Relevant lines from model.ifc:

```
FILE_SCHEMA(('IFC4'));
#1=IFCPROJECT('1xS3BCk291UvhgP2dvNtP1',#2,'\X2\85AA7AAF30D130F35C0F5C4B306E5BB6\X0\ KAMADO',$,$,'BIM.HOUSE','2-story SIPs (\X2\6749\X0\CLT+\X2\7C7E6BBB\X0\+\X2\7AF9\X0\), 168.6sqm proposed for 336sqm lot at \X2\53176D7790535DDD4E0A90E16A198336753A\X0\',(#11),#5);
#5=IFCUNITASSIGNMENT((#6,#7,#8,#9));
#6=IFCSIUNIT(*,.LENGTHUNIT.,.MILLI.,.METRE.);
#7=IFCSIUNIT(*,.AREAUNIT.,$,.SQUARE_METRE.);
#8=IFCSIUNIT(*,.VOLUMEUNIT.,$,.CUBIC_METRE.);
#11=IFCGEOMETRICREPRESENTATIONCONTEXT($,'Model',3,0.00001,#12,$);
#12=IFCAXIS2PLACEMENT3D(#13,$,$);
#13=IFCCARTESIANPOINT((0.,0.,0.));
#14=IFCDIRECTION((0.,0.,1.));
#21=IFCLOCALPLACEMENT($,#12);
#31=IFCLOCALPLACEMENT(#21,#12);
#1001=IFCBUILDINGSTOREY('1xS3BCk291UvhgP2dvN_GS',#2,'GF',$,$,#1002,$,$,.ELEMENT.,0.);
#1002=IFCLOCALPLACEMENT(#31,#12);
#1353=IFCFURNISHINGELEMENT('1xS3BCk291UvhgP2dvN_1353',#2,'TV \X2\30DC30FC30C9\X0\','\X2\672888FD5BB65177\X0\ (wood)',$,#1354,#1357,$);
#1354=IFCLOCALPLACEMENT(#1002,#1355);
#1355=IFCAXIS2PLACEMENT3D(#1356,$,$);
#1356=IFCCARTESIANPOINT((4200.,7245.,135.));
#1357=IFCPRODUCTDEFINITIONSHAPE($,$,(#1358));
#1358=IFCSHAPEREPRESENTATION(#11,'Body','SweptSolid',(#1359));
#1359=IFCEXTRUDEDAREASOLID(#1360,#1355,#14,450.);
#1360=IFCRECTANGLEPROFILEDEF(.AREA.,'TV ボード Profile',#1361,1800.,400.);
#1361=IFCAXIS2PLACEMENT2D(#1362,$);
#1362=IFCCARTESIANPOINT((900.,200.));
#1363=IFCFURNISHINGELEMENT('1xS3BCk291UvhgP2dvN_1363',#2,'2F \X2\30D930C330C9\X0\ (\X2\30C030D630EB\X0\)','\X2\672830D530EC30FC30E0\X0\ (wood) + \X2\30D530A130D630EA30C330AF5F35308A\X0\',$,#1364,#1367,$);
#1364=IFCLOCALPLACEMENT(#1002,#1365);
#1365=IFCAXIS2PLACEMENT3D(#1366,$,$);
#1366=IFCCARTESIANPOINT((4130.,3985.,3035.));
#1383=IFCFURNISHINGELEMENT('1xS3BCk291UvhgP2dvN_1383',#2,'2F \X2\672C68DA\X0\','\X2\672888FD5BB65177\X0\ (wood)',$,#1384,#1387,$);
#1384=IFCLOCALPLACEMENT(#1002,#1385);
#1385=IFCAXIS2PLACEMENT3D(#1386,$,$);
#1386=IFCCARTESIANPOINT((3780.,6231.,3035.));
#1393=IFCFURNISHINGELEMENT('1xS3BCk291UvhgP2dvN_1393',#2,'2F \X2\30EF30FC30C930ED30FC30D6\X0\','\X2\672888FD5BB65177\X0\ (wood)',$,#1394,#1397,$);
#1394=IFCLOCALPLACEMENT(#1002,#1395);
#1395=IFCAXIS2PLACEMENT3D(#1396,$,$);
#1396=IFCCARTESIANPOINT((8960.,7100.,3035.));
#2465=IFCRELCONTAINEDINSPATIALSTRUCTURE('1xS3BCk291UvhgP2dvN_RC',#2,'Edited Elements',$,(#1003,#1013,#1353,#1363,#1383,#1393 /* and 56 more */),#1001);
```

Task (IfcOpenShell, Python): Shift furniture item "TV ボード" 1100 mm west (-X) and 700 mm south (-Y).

```python
import ifcopenshell
import ifcopenshell.api.geometry
import ifcopenshell.util.placement

model = ifcopenshell.open("model.ifc")

item = model.by_guid("1xS3BCk291UvhgP2dvN_1353")
matrix = ifcopenshell.util.placement.get_local_placement(item.ObjectPlacement)
matrix[0, 3] -= 1100.0
matrix[1, 3] -= 700.0
ifcopenshell.api.geometry.edit_object_placement(model, product=item, matrix=matrix, is_si=False)

print(ifcopenshell.util.placement.get_local_placement(item.ObjectPlacement).round(3) + 0.0)

model.write("model_rev.ifc")
```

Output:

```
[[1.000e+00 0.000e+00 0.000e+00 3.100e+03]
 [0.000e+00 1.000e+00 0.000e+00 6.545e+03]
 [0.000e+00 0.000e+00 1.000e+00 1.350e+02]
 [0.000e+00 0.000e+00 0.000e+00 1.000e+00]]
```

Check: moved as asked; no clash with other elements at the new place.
